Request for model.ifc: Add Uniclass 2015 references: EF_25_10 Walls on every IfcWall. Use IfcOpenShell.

First a look at what the model holds.

```python
import ifcopenshell

model = ifcopenshell.open("model.ifc")
print(model.schema)
print("classifications:", [c.Name for c in model.by_type("IfcClassification")])
for ifc_class in ("IfcDoor", "IfcRoof", "IfcStair", "IfcWall", "IfcWindow"):
    print(ifc_class, len(model.by_type(ifc_class)))
```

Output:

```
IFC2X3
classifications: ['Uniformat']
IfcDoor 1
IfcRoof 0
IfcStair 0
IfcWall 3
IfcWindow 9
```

```python
import ifcopenshell
import ifcopenshell.api.classification

model = ifcopenshell.open("model.ifc")

# IFC2X3 requires Source and Edition and has no link from the project to the system.
system = model.create_entity("IfcClassification", Source="NBS", Edition="2015", Name="Uniclass 2015")

codes = {
    "IfcWall": ("EF_25_10", "Walls"),
}
for ifc_class, (code, name) in codes.items():
    products = model.by_type(ifc_class)
    ifcopenshell.api.classification.add_reference(
        model, products=products, classification=system, identification=code, name=name
    )
    print(code, len(products))

model.write("model_rev.ifc")
```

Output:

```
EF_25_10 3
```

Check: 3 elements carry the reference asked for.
